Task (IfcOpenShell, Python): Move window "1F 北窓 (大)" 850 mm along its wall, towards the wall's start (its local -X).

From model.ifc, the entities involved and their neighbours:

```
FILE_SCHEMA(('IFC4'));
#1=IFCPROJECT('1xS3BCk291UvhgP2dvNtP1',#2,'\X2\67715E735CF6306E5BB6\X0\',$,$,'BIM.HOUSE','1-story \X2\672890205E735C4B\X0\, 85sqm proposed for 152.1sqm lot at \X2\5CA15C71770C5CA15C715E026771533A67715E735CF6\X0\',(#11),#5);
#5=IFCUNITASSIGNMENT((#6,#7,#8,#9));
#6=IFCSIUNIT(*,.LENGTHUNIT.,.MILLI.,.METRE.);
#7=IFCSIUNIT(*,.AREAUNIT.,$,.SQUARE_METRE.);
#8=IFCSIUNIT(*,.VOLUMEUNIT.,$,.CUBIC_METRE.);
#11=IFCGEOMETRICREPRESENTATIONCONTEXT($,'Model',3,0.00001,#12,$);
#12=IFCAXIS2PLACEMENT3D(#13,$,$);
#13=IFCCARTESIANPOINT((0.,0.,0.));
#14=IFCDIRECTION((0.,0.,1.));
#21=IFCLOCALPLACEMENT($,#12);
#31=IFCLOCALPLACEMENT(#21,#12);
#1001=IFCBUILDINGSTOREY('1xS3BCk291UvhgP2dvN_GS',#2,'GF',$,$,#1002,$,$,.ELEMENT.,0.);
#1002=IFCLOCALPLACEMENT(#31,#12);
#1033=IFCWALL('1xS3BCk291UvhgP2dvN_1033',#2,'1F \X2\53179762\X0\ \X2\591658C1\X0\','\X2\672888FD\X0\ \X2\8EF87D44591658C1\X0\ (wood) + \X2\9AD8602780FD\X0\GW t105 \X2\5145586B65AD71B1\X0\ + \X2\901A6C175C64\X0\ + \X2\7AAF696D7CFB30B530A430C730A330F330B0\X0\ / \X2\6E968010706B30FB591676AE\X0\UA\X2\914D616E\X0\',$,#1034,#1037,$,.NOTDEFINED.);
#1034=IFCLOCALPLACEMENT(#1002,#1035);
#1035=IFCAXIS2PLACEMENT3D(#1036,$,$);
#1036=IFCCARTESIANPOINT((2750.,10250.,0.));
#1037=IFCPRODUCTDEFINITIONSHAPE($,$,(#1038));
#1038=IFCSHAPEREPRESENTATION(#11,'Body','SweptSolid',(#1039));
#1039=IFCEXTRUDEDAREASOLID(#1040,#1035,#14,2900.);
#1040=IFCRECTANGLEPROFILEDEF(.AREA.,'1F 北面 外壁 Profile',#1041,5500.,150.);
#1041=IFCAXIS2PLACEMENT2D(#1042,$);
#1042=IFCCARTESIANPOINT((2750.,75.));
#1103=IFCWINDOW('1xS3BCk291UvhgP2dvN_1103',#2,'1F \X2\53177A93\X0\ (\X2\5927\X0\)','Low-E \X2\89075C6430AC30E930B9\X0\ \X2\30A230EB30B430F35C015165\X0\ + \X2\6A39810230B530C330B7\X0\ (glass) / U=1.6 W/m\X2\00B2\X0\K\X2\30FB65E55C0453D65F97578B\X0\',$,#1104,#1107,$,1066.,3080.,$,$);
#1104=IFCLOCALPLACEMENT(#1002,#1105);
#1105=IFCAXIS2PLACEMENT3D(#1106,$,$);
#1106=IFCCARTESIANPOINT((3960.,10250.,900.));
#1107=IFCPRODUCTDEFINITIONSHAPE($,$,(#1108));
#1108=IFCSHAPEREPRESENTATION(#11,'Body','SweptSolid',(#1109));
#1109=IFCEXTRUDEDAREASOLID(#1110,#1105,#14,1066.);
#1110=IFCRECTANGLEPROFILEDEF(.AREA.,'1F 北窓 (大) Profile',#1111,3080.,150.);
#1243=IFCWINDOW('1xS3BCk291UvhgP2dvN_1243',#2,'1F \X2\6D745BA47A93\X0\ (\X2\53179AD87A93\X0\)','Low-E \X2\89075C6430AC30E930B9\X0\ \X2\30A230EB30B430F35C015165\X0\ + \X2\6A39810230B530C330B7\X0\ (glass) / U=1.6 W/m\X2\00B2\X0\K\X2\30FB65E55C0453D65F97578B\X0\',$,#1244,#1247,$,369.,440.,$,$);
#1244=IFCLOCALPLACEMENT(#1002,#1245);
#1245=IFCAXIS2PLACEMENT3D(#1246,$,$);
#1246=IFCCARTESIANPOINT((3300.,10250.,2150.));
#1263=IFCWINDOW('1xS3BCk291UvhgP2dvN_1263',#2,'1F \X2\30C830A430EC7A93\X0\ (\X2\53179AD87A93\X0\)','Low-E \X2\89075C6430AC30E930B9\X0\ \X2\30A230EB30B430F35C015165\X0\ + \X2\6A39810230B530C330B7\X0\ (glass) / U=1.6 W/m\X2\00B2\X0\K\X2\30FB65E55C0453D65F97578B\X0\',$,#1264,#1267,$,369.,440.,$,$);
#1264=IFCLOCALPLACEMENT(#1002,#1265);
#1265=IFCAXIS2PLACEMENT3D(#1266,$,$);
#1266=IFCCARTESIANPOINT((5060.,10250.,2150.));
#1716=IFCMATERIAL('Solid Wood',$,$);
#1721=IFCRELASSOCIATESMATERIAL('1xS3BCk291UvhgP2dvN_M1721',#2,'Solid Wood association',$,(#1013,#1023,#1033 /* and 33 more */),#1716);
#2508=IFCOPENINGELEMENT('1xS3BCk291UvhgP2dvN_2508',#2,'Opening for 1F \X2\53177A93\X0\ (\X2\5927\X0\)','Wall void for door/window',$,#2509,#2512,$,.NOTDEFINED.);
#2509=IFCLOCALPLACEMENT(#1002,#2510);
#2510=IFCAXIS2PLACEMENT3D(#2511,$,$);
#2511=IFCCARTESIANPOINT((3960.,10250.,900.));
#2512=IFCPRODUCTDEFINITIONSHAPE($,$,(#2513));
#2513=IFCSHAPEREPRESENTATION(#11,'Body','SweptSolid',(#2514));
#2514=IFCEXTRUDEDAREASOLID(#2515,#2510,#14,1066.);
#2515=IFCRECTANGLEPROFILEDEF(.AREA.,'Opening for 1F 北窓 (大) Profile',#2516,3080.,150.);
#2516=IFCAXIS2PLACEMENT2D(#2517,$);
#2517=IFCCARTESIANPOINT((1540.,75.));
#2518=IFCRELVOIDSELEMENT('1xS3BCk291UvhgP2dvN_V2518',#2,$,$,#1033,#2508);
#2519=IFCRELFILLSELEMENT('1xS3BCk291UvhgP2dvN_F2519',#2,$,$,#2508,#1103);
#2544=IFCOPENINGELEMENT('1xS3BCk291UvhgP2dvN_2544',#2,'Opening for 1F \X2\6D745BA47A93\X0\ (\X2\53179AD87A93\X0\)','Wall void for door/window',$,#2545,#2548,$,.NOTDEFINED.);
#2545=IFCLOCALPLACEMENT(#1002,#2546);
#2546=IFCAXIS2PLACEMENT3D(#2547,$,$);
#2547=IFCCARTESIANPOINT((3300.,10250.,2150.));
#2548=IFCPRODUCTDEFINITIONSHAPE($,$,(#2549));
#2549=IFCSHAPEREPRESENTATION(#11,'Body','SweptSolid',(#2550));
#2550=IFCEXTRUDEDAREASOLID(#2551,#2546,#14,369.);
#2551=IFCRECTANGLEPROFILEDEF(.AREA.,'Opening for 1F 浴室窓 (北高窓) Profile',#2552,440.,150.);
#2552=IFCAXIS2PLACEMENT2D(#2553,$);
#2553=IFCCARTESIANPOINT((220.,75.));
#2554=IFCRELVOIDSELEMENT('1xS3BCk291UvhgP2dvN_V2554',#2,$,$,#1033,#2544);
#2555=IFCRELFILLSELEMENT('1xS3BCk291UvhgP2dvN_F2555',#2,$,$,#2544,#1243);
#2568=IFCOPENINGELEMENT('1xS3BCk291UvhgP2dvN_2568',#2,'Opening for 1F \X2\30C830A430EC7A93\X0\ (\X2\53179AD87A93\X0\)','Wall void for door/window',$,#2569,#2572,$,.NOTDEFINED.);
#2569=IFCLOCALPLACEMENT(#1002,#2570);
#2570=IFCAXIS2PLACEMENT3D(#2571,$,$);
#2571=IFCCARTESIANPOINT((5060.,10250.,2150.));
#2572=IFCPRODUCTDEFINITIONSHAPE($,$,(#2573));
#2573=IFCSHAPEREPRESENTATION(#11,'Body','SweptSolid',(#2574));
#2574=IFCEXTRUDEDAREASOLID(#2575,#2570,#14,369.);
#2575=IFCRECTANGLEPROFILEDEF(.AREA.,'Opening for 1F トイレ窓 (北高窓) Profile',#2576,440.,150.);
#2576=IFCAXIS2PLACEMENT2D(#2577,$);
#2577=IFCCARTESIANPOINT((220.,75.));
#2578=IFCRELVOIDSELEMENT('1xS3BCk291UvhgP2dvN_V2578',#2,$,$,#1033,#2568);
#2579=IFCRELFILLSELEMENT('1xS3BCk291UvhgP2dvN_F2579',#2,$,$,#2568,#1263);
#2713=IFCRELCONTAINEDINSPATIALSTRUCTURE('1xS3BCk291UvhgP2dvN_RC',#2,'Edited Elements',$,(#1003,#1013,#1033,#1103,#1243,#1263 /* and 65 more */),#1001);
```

```python
import ifcopenshell
import ifcopenshell.api.geometry
import ifcopenshell.util.placement
import ifcopenshell.util.unit

model = ifcopenshell.open("model.ifc")
unit_scale = ifcopenshell.util.unit.calculate_unit_scale(model)

window = model.by_guid("1xS3BCk291UvhgP2dvN_1103")
opening = window.FillsVoids[0].RelatingOpeningElement
wall = opening.VoidsElements[0].RelatingBuildingElement

wall_matrix = ifcopenshell.util.placement.get_local_placement(wall.ObjectPlacement)
shift = wall_matrix[:3, 0] * -0.85 / unit_scale
before = ifcopenshell.util.placement.get_local_placement(window.ObjectPlacement)[:3, 3].copy()

# The window is not placed relative to its opening, so move both.
for product in (opening, window):
    matrix = ifcopenshell.util.placement.get_local_placement(product.ObjectPlacement)
    matrix[:3, 3] += shift
    ifcopenshell.api.geometry.edit_object_placement(model, product=product, matrix=matrix, is_si=False)

after = ifcopenshell.util.placement.get_local_placement(window.ObjectPlacement)[:3, 3]
print("window moved by", (after - before).round(3) + 0.0)

model.write("model-out.ifc")
```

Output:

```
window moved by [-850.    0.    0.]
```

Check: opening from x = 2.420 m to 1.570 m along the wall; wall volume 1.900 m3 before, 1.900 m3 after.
